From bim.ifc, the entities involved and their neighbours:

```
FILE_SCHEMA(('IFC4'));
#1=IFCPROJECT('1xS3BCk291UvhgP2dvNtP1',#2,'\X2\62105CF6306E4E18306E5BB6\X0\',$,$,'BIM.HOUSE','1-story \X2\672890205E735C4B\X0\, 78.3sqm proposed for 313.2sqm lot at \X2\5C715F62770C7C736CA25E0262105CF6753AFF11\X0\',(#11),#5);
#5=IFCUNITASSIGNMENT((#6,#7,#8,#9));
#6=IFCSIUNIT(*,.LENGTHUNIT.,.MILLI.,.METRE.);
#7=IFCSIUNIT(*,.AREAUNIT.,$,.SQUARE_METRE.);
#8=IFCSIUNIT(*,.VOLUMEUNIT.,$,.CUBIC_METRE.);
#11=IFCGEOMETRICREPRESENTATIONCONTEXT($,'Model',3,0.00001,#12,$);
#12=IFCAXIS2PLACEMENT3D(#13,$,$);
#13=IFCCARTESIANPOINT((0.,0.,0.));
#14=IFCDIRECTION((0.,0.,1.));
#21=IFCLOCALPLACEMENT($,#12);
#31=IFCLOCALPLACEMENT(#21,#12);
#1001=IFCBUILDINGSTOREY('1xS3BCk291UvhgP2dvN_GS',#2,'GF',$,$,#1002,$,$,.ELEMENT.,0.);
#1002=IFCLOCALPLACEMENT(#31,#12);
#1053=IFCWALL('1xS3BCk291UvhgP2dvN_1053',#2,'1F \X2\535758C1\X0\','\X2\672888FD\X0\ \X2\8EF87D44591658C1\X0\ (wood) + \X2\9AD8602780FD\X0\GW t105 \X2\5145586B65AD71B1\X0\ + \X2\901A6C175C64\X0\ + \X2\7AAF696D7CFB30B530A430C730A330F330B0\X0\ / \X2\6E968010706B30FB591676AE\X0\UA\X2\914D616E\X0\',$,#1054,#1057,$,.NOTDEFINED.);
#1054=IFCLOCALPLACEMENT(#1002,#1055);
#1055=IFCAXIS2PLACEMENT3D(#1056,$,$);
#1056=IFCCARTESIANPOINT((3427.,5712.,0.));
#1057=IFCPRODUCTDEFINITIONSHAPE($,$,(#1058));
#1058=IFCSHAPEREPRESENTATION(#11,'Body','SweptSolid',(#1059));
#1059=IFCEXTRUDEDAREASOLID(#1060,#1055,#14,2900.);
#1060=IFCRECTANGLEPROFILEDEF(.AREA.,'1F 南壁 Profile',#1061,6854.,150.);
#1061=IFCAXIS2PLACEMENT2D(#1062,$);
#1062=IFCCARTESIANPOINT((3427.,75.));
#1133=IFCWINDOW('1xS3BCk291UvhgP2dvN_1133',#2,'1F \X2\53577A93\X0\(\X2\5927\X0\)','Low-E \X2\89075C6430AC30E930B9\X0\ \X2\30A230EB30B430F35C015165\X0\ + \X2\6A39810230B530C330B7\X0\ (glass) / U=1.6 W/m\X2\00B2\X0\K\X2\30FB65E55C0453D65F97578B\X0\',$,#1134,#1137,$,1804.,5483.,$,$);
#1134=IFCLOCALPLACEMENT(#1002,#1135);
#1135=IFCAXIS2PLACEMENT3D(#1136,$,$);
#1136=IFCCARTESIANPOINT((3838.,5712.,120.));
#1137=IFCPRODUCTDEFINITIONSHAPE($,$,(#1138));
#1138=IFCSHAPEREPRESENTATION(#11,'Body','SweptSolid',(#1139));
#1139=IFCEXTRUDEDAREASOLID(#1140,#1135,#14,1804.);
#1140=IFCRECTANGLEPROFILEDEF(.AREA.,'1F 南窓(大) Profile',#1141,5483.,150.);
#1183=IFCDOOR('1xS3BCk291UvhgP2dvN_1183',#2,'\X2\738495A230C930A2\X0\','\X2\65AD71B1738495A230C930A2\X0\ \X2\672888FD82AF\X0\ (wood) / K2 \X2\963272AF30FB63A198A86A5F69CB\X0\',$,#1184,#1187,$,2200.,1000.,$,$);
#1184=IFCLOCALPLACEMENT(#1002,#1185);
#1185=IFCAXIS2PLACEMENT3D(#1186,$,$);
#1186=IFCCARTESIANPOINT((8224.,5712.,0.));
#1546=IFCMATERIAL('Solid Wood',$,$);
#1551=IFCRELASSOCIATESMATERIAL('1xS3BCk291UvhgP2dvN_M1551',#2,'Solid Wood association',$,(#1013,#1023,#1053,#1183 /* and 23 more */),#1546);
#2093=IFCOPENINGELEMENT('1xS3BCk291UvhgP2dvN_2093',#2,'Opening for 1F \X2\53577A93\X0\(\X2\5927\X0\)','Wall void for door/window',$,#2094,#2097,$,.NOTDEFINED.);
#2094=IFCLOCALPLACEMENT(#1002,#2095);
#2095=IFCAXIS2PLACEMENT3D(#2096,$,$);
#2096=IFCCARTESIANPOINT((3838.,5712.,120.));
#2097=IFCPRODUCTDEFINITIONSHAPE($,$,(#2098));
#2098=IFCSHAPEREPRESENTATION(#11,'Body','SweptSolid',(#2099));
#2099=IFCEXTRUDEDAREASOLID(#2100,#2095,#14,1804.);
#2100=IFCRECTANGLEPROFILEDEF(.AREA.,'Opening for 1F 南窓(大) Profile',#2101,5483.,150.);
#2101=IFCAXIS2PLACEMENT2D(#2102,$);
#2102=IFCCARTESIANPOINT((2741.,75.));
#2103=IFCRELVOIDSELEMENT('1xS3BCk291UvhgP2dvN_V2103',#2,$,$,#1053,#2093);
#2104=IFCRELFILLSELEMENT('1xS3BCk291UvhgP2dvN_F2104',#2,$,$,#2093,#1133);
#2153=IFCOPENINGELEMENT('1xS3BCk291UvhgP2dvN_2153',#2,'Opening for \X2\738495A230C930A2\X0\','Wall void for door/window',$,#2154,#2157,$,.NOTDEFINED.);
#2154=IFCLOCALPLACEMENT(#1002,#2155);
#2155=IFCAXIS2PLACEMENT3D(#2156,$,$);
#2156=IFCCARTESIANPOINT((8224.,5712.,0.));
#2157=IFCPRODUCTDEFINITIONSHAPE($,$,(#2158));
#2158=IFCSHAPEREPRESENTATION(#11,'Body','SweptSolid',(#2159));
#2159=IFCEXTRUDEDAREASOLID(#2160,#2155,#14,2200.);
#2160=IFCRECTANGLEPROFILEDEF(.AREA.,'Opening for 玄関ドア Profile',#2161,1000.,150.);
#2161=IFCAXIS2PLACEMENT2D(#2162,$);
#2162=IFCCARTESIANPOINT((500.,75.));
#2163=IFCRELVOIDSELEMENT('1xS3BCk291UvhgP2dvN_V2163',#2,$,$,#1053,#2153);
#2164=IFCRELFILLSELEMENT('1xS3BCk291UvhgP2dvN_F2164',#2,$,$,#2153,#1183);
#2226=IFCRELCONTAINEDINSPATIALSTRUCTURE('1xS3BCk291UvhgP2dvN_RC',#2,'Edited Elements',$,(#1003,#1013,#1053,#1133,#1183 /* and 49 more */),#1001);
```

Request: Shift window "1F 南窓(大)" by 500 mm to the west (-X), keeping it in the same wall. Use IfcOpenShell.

```python
import ifcopenshell
import ifcopenshell.api.geometry
import ifcopenshell.util.placement
import ifcopenshell.util.unit

model = ifcopenshell.open("bim.ifc")
unit_scale = ifcopenshell.util.unit.calculate_unit_scale(model)

window = model.by_guid("1xS3BCk291UvhgP2dvN_1133")
opening = window.FillsVoids[0].RelatingOpeningElement
wall = opening.VoidsElements[0].RelatingBuildingElement

wall_matrix = ifcopenshell.util.placement.get_local_placement(wall.ObjectPlacement)
shift = wall_matrix[:3, 0] * -0.5 / unit_scale
before = ifcopenshell.util.placement.get_local_placement(window.ObjectPlacement)[:3, 3].copy()

# The window is not placed relative to its opening, so move both.
for product in (opening, window):
    matrix = ifcopenshell.util.placement.get_local_placement(product.ObjectPlacement)
    matrix[:3, 3] += shift
    ifcopenshell.api.geometry.edit_object_placement(model, product=product, matrix=matrix, is_si=False)

after = ifcopenshell.util.placement.get_local_placement(window.ObjectPlacement)[:3, 3]
print("window moved by", (after - before).round(3) + 0.0)

model.write("bim-out.ifc")
```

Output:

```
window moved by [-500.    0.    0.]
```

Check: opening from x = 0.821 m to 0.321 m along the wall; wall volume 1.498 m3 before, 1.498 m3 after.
